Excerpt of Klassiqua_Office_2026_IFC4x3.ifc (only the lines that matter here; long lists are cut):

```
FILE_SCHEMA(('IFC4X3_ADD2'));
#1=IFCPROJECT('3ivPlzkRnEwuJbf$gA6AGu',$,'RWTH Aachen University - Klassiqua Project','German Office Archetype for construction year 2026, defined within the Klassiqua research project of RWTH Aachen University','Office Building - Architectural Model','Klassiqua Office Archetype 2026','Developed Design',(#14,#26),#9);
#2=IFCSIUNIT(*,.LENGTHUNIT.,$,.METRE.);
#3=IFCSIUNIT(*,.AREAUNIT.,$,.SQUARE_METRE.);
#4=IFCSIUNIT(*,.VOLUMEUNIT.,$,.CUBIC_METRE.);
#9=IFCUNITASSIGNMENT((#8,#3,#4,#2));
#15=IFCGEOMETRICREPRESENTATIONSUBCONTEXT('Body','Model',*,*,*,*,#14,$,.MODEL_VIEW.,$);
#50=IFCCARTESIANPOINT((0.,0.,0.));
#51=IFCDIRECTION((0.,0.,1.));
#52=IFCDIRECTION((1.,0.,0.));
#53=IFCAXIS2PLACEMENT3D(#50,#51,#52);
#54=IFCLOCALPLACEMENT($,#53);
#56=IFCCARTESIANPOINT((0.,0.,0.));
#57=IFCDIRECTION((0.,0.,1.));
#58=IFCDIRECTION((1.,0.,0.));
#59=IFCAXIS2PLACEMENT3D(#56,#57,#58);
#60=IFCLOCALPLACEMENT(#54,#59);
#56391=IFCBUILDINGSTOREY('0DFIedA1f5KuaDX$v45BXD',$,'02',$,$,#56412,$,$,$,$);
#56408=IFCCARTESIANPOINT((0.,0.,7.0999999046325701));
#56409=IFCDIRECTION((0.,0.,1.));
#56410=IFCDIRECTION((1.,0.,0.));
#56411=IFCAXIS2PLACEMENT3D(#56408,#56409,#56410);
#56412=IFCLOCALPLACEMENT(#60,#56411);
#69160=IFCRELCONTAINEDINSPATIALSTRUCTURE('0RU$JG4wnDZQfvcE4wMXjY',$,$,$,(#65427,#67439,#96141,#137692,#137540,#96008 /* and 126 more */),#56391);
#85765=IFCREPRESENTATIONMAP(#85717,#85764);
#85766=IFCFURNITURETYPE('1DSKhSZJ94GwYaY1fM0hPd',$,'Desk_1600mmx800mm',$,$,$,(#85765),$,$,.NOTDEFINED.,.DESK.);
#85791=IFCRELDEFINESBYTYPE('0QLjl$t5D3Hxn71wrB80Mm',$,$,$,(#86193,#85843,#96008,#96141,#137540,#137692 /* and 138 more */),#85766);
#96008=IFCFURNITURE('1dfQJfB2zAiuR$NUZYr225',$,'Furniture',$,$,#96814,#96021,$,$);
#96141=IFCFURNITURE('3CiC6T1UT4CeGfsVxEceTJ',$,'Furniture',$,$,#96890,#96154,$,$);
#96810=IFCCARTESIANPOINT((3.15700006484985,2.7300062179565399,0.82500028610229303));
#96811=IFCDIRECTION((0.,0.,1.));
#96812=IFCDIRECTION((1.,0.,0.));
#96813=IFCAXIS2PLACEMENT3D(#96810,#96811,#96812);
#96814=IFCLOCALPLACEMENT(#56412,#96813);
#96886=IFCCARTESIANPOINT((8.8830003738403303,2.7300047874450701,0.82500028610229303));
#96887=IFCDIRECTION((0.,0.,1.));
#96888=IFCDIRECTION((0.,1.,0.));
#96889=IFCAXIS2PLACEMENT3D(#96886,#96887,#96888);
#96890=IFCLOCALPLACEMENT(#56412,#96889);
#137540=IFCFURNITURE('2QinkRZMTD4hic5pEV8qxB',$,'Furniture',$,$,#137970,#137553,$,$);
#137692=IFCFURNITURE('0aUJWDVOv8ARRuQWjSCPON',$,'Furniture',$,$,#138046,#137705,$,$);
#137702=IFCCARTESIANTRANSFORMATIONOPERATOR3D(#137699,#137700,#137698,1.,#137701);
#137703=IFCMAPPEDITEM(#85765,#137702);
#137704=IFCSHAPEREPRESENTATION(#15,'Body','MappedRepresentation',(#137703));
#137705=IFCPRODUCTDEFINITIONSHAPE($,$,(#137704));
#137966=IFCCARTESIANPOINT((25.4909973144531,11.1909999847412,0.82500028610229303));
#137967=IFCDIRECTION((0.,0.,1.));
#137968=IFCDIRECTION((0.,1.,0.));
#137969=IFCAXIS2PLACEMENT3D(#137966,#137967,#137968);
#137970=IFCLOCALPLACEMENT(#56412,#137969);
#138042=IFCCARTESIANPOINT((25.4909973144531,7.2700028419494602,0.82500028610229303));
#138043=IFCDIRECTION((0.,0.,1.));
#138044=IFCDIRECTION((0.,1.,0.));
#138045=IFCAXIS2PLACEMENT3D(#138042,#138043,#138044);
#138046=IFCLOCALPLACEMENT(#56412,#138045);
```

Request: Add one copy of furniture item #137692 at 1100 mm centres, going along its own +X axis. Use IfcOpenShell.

```python
import ifcopenshell
import ifcopenshell.api.geometry
import ifcopenshell.api.root
import ifcopenshell.util.element
import ifcopenshell.util.placement
import ifcopenshell.util.unit

model = ifcopenshell.open("Klassiqua_Office_2026_IFC4x3.ifc")
unit_scale = ifcopenshell.util.unit.calculate_unit_scale(model)

source = model.by_id(137692)
base = ifcopenshell.util.placement.get_local_placement(source.ObjectPlacement)
step = base[:3, 0] * 1.1 / unit_scale

for i in range(1, 2):
    copy = ifcopenshell.api.root.copy_class(model, product=source)
    copy.Representation = ifcopenshell.util.element.copy_deep(
        model, source.Representation, exclude=["IfcGeometricRepresentationContext", "IfcRepresentationMap"]
    )
    matrix = base.copy()
    matrix[:3, 3] += i * step
    print("added at", matrix[:3, 3].round(3) + 0.0)
    ifcopenshell.api.geometry.edit_object_placement(model, product=copy, matrix=matrix, is_si=False)

model.write("Klassiqua_Office_2026_IFC4x3_rev.ifc")
```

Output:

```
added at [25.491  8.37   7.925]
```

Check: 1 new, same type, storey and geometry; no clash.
